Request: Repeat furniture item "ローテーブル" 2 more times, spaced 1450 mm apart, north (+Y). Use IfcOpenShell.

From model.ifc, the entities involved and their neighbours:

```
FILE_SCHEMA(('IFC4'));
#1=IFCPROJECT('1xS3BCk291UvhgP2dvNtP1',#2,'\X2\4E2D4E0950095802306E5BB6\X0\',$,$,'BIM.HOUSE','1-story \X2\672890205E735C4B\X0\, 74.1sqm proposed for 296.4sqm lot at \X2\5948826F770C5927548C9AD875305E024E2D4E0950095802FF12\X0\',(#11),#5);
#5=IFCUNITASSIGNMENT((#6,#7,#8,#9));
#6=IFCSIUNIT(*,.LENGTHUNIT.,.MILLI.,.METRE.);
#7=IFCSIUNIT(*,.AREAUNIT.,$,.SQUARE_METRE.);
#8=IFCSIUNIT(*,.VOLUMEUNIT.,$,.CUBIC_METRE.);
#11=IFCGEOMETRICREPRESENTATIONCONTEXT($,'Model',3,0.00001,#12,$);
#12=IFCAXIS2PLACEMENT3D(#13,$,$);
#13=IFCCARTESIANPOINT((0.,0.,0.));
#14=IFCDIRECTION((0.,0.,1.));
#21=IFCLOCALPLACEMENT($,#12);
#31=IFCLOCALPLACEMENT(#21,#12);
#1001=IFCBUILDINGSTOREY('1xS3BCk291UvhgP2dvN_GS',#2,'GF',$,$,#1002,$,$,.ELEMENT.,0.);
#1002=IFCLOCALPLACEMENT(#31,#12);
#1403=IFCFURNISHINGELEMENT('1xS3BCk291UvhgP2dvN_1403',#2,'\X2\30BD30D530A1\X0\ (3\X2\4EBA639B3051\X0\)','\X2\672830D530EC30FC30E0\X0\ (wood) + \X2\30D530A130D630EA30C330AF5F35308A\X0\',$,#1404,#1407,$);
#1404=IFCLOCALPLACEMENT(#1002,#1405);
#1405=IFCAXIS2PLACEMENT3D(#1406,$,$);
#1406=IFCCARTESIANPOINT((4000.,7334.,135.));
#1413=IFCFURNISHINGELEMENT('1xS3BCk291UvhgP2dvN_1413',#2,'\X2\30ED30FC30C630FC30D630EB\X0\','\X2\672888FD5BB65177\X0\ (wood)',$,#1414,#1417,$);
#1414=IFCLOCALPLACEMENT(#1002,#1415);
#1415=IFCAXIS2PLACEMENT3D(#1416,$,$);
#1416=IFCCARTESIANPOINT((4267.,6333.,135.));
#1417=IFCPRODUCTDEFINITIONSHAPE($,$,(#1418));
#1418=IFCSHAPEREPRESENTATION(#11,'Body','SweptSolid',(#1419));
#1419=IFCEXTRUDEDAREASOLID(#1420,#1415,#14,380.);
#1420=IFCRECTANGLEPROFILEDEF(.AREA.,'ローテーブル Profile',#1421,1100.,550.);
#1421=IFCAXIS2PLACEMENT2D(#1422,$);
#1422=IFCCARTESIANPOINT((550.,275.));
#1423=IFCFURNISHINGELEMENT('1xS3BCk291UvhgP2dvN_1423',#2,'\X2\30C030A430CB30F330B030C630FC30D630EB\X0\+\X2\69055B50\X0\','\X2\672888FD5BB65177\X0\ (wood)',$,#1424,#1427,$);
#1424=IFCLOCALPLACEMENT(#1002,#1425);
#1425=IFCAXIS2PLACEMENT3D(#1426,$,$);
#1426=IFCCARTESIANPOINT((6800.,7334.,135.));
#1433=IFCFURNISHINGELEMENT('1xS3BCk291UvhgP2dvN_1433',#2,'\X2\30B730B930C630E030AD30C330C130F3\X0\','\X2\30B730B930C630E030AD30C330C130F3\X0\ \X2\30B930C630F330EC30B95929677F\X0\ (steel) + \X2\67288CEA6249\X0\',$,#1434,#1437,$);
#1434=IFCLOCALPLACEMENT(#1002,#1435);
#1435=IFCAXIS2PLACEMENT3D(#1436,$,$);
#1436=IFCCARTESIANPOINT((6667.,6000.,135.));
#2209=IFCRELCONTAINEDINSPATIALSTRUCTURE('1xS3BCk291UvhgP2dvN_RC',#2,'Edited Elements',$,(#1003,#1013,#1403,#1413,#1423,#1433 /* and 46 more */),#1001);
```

```python
import numpy as np
import ifcopenshell
import ifcopenshell.api.geometry
import ifcopenshell.api.root
import ifcopenshell.util.element
import ifcopenshell.util.placement
import ifcopenshell.util.unit

model = ifcopenshell.open("model.ifc")
unit_scale = ifcopenshell.util.unit.calculate_unit_scale(model)


def reuse_history(source, copy):
    """copy_class also copies each property set's owner history, people and application; keep the originals."""
    for rel in copy.IsDefinedBy:
        if rel.is_a("IfcRelDefinesByProperties") and (history := rel.RelatingPropertyDefinition.OwnerHistory):
            rel.RelatingPropertyDefinition.OwnerHistory = source.OwnerHistory
            ifcopenshell.util.element.remove_deep2(model, history)


source = model.by_guid("1xS3BCk291UvhgP2dvN_1413")
base = ifcopenshell.util.placement.get_local_placement(source.ObjectPlacement)
step = np.array([0.0, 1.0, 0.0]) * 1.45 / unit_scale

for i in range(1, 3):
    copy = ifcopenshell.api.root.copy_class(model, product=source)
    copy.Representation = ifcopenshell.util.element.copy_deep(
        model, source.Representation, exclude=["IfcGeometricRepresentationContext", "IfcRepresentationMap"]
    )
    reuse_history(source, copy)
    matrix = base.copy()
    matrix[:3, 3] += i * step
    print("added at", matrix[:3, 3].round(3) + 0.0)
    ifcopenshell.api.geometry.edit_object_placement(model, product=copy, matrix=matrix, is_si=False)

model.write("model_rev.ifc")
```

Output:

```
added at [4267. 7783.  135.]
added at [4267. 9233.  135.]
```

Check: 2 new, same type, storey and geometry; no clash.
